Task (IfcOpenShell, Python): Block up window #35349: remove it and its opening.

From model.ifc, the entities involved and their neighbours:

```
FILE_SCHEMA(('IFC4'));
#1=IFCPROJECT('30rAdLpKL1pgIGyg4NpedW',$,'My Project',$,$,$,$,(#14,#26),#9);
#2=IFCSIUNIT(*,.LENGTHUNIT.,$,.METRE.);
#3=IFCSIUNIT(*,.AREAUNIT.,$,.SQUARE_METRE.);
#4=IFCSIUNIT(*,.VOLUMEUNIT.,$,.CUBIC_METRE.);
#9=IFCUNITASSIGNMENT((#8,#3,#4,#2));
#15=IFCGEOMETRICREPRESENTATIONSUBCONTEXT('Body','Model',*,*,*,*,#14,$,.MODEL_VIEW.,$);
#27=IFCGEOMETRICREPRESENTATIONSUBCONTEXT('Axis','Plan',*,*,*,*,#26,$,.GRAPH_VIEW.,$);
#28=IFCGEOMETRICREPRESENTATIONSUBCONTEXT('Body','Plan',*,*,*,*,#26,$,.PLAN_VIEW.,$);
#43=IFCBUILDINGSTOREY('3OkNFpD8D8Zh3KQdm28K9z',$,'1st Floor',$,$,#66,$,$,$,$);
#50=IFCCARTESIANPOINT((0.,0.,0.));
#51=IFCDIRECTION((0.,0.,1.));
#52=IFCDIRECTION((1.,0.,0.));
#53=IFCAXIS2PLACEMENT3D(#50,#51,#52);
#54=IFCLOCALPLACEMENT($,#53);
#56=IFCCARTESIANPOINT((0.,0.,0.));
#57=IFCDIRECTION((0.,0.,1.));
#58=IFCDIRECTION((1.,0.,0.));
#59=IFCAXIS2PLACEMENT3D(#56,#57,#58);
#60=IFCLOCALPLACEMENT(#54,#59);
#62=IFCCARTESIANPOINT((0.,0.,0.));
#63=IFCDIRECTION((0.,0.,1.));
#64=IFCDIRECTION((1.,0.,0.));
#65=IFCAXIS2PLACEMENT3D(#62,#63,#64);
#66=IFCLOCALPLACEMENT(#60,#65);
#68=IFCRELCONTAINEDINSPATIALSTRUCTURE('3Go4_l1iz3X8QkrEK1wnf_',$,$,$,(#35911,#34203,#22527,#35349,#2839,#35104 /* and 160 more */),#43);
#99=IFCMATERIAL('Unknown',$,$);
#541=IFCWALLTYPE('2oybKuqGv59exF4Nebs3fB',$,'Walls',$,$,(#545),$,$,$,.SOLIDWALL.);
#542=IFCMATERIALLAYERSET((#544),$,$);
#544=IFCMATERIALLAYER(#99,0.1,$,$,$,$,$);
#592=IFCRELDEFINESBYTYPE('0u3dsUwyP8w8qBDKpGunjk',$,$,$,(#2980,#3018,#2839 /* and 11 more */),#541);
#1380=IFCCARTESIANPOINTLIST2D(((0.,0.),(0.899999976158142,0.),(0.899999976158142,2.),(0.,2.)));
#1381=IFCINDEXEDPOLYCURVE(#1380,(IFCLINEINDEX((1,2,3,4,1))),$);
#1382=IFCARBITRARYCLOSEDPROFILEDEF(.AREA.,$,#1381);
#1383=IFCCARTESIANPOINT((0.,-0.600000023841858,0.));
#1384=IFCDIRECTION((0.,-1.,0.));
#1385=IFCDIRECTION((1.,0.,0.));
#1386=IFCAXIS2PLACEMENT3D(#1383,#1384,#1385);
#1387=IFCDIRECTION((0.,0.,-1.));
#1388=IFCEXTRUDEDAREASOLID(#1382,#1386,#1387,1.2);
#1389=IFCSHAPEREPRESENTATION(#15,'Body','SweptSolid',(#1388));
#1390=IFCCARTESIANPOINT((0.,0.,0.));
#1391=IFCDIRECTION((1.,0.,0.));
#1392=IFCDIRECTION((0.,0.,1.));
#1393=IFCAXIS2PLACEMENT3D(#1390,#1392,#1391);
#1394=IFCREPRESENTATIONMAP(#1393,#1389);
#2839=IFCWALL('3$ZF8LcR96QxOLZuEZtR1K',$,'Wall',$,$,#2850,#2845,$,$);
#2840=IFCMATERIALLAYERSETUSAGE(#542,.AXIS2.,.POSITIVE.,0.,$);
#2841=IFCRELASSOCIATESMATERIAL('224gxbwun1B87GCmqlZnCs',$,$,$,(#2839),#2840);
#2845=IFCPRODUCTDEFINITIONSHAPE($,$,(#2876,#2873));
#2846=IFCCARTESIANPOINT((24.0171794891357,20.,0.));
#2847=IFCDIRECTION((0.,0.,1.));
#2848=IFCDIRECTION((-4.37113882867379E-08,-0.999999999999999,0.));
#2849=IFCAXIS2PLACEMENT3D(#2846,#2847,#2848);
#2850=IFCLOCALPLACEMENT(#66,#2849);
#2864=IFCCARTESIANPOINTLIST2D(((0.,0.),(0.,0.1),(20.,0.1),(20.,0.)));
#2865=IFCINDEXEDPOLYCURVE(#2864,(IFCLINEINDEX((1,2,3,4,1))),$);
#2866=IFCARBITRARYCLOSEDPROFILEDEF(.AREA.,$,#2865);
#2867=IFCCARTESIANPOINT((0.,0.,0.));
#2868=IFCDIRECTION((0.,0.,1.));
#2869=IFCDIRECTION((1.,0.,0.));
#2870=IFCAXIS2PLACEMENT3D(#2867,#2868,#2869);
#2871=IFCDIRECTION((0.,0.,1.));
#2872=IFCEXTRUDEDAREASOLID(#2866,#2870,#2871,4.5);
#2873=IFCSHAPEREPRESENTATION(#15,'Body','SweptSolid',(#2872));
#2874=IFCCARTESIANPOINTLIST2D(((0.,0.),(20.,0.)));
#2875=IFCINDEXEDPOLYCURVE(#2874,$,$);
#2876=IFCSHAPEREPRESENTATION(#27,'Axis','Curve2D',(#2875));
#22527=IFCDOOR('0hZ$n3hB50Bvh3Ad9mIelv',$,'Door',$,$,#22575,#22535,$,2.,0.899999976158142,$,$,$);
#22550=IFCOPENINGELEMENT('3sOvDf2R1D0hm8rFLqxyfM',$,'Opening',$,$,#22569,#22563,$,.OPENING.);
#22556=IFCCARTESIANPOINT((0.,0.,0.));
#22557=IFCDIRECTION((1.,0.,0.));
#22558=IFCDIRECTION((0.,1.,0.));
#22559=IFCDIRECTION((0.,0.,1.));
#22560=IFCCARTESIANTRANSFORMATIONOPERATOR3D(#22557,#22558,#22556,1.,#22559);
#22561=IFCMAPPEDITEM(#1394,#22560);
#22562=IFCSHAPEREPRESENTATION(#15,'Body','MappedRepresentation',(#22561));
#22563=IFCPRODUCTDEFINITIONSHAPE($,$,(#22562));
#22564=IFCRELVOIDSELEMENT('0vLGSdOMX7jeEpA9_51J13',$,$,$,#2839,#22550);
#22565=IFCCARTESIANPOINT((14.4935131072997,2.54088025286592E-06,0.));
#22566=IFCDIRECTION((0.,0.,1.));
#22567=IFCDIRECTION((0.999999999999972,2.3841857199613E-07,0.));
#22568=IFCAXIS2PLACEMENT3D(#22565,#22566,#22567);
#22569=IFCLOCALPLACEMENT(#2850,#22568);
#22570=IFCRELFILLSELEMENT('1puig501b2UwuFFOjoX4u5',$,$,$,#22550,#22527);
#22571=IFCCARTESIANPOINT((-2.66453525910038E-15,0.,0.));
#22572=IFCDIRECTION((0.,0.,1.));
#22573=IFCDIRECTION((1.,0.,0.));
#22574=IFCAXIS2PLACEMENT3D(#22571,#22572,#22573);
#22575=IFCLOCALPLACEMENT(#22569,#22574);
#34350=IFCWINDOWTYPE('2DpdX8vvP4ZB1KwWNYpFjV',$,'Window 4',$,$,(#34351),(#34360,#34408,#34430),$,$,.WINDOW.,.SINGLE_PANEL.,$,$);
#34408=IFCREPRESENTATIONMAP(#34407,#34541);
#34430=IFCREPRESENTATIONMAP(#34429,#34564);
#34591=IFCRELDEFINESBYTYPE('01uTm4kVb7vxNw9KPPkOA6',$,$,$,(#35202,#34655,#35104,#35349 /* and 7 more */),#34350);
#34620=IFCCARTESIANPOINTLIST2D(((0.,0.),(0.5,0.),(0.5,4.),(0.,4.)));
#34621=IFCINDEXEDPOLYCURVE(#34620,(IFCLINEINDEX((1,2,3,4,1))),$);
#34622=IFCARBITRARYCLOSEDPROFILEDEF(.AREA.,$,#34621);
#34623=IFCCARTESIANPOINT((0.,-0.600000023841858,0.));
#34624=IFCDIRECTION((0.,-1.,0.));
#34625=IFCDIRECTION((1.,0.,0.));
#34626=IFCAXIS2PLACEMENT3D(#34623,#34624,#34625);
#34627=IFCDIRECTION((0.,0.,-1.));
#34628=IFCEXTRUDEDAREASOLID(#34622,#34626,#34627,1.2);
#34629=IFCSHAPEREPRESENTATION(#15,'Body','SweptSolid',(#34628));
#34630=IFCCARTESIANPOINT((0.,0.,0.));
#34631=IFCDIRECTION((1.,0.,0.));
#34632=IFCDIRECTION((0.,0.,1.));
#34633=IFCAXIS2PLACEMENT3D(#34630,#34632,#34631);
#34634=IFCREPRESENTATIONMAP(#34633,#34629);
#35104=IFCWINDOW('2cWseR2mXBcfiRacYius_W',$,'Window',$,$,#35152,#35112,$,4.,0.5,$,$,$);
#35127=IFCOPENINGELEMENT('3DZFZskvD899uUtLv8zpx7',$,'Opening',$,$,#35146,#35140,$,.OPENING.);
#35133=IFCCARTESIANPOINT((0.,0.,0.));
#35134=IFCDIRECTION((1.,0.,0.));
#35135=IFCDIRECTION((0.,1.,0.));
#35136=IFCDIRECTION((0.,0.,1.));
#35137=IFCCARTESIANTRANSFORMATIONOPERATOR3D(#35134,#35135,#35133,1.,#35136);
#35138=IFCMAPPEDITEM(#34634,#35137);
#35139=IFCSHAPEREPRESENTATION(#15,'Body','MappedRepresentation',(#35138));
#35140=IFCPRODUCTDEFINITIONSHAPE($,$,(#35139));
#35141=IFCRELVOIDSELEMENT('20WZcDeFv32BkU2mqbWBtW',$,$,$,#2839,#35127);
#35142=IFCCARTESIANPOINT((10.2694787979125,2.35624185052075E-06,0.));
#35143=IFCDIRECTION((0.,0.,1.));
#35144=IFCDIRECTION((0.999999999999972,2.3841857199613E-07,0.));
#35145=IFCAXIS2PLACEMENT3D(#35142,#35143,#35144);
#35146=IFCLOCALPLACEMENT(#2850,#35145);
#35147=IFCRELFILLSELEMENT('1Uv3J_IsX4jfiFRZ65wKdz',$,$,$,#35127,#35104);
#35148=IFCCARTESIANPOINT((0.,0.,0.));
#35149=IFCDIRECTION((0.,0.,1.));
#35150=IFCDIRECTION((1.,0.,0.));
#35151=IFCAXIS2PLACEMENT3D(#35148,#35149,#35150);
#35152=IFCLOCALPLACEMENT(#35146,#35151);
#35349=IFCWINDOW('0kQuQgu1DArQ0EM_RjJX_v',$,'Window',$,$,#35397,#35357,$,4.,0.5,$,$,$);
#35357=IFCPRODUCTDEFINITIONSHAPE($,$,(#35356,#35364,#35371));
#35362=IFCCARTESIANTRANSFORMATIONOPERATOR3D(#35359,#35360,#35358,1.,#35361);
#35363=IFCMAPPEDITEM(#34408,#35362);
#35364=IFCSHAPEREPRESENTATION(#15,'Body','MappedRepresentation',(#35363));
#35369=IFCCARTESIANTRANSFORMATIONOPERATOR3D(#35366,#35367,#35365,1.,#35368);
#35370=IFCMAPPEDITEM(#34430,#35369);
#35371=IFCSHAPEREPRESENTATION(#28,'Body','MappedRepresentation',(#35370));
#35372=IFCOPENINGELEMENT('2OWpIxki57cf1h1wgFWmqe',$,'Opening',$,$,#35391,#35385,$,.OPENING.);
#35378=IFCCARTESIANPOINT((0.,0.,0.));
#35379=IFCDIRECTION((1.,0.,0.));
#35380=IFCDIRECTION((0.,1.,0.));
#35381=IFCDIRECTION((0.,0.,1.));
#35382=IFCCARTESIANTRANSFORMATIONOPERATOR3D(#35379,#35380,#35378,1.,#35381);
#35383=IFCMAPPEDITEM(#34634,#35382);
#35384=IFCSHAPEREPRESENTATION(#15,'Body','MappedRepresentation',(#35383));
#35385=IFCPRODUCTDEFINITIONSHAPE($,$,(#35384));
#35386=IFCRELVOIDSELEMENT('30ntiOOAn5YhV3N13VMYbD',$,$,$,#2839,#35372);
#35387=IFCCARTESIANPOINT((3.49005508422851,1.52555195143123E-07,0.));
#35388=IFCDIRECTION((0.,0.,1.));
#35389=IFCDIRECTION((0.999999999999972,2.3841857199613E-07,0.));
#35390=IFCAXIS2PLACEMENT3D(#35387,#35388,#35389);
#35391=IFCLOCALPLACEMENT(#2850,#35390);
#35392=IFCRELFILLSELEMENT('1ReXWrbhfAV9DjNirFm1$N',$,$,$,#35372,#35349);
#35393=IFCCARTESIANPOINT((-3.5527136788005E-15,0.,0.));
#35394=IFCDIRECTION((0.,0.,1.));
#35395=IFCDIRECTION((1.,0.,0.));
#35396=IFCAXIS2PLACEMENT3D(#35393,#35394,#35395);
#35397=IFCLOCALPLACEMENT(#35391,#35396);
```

```python
import ifcopenshell
import ifcopenshell.api.feature
import ifcopenshell.api.root
import ifcopenshell.geom
import ifcopenshell.util.shape

model = ifcopenshell.open("model.ifc")
settings = ifcopenshell.geom.settings()


def volume(element):
    """Net volume in cubic metres, openings subtracted."""
    shape = ifcopenshell.geom.create_shape(settings, element)
    return ifcopenshell.util.shape.get_volume(shape.geometry)


window = model.by_id(35349)
opening = window.FillsVoids[0].RelatingOpeningElement
wall = opening.VoidsElements[0].RelatingBuildingElement
before = volume(wall)

ifcopenshell.api.root.remove_product(model, product=window)
ifcopenshell.api.feature.remove_feature(model, feature=opening)

after = volume(wall)

print(f"wall volume {before:.3f} -> {after:.3f} m3")

model.write("model-out.ifc")
```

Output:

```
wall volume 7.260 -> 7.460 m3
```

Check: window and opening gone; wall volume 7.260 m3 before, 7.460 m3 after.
